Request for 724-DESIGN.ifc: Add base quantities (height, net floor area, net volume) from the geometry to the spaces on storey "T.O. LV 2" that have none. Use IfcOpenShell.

First a look at what the model holds.

```python
import ifcopenshell
import ifcopenshell.util.element
import ifcopenshell.util.unit

model = ifcopenshell.open("724-DESIGN.ifc")
print(model.schema)
for unit_type in ("LENGTHUNIT", "AREAUNIT", "VOLUMEUNIT"):
    print(unit_type, ifcopenshell.util.unit.calculate_unit_scale(model, unit_type))
storey = next(s for s in model.by_type("IfcBuildingStorey") if s.Name == "T.O. LV 2")
spaces = [e for e in ifcopenshell.util.element.get_decomposition(storey) if e.is_a("IfcSpace")]
for e in sorted(spaces, key=lambda e: e.id()):
    print(e.id(), e.is_a(), e.Name, list(ifcopenshell.util.element.get_psets(e, qtos_only=True)), sep=" | ")
```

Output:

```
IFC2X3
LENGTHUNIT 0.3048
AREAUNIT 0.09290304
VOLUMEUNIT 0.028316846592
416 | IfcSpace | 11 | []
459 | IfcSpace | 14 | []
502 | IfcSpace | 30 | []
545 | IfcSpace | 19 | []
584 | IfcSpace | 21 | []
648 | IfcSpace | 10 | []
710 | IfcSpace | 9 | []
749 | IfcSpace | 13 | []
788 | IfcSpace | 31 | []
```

```python
import ifcopenshell
import ifcopenshell.api.pset
import ifcopenshell.geom
import ifcopenshell.util.element
import ifcopenshell.util.shape
import ifcopenshell.util.unit

model = ifcopenshell.open("724-DESIGN.ifc")
unit_scale = ifcopenshell.util.unit.calculate_unit_scale(model)
area_scale = ifcopenshell.util.unit.calculate_unit_scale(model, "AREAUNIT")
volume_scale = ifcopenshell.util.unit.calculate_unit_scale(model, "VOLUMEUNIT")
settings = ifcopenshell.geom.settings()

storey = next(s for s in model.by_type("IfcBuildingStorey") if s.Name == "T.O. LV 2")
spaces = [e for e in ifcopenshell.util.element.get_decomposition(storey) if e.is_a("IfcSpace")]

for e in sorted(spaces, key=lambda e: e.id()):
    if ifcopenshell.util.element.get_psets(e, qtos_only=True, should_inherit=False):
        continue
    # Geometry comes back in metres, in the element's own axes.
    shape = ifcopenshell.geom.create_shape(settings, e)
    values = {
        "Height": ifcopenshell.util.shape.get_z(shape.geometry) / unit_scale,
        "NetFloorArea": ifcopenshell.util.shape.get_footprint_area(shape.geometry) / area_scale,
        "NetVolume": ifcopenshell.util.shape.get_volume(shape.geometry) / volume_scale,
    }
    qto = ifcopenshell.api.pset.add_qto(model, product=e, name="BaseQuantities")
    ifcopenshell.api.pset.edit_qto(model, qto=qto, properties=values)
    print(e.id(), {k: round(v, 3) for k, v in values.items()})

model.write("724-DESIGN-out.ifc")
```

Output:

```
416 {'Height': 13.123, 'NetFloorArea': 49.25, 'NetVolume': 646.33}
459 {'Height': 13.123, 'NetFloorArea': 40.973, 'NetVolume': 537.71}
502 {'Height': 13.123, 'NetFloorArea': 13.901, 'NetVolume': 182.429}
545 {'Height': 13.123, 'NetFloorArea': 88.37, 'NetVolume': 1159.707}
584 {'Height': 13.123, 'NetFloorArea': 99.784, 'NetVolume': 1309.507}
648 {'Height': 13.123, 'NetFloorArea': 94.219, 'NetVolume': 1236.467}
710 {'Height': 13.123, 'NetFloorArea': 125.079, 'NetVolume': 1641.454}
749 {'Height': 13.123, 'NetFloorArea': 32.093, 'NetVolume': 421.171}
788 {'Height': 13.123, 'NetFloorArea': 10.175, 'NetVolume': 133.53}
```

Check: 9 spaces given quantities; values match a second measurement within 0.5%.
